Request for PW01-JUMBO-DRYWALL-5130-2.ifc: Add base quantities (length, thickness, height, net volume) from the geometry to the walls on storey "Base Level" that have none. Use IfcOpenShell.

First a look at what the model holds.

```python
import ifcopenshell
import ifcopenshell.util.element
import ifcopenshell.util.unit

model = ifcopenshell.open("PW01-JUMBO-DRYWALL-5130-2.ifc")
print(model.schema)
for unit_type in ("LENGTHUNIT", "AREAUNIT", "VOLUMEUNIT"):
    print(unit_type, ifcopenshell.util.unit.calculate_unit_scale(model, unit_type))
storey = next(s for s in model.by_type("IfcBuildingStorey") if s.Name == "Base Level")
walls = [e for e in ifcopenshell.util.element.get_decomposition(storey) if e.is_a("IfcWall")]
for e in sorted(walls, key=lambda e: e.id()):
    print(e.id(), e.is_a(), e.Name, list(ifcopenshell.util.element.get_psets(e, qtos_only=True)), sep=" | ")
```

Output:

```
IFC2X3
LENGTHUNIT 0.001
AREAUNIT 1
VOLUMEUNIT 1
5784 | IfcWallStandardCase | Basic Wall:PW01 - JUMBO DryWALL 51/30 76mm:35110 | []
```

```python
import ifcopenshell
import ifcopenshell.api.pset
import ifcopenshell.geom
import ifcopenshell.util.element
import ifcopenshell.util.shape
import ifcopenshell.util.unit

model = ifcopenshell.open("PW01-JUMBO-DRYWALL-5130-2.ifc")
unit_scale = ifcopenshell.util.unit.calculate_unit_scale(model)
volume_scale = ifcopenshell.util.unit.calculate_unit_scale(model, "VOLUMEUNIT")
settings = ifcopenshell.geom.settings()

storey = next(s for s in model.by_type("IfcBuildingStorey") if s.Name == "Base Level")
walls = [e for e in ifcopenshell.util.element.get_decomposition(storey) if e.is_a("IfcWall")]

for e in sorted(walls, key=lambda e: e.id()):
    if ifcopenshell.util.element.get_psets(e, qtos_only=True, should_inherit=False):
        continue
    # Geometry comes back in metres, in the element's own axes.
    shape = ifcopenshell.geom.create_shape(settings, e)
    values = {
        "Length": ifcopenshell.util.shape.get_x(shape.geometry) / unit_scale,
        "Width": ifcopenshell.util.shape.get_y(shape.geometry) / unit_scale,
        "Height": ifcopenshell.util.shape.get_z(shape.geometry) / unit_scale,
        "NetVolume": ifcopenshell.util.shape.get_volume(shape.geometry) / volume_scale,
    }
    qto = ifcopenshell.api.pset.add_qto(model, product=e, name="BaseQuantities")
    ifcopenshell.api.pset.edit_qto(model, qto=qto, properties=values)
    print(e.id(), {k: round(v, 3) for k, v in values.items()})

model.write("PW01-JUMBO-DRYWALL-5130-2_rev.ifc")
```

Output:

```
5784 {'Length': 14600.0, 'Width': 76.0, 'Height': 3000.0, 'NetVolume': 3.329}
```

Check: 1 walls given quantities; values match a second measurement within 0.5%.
